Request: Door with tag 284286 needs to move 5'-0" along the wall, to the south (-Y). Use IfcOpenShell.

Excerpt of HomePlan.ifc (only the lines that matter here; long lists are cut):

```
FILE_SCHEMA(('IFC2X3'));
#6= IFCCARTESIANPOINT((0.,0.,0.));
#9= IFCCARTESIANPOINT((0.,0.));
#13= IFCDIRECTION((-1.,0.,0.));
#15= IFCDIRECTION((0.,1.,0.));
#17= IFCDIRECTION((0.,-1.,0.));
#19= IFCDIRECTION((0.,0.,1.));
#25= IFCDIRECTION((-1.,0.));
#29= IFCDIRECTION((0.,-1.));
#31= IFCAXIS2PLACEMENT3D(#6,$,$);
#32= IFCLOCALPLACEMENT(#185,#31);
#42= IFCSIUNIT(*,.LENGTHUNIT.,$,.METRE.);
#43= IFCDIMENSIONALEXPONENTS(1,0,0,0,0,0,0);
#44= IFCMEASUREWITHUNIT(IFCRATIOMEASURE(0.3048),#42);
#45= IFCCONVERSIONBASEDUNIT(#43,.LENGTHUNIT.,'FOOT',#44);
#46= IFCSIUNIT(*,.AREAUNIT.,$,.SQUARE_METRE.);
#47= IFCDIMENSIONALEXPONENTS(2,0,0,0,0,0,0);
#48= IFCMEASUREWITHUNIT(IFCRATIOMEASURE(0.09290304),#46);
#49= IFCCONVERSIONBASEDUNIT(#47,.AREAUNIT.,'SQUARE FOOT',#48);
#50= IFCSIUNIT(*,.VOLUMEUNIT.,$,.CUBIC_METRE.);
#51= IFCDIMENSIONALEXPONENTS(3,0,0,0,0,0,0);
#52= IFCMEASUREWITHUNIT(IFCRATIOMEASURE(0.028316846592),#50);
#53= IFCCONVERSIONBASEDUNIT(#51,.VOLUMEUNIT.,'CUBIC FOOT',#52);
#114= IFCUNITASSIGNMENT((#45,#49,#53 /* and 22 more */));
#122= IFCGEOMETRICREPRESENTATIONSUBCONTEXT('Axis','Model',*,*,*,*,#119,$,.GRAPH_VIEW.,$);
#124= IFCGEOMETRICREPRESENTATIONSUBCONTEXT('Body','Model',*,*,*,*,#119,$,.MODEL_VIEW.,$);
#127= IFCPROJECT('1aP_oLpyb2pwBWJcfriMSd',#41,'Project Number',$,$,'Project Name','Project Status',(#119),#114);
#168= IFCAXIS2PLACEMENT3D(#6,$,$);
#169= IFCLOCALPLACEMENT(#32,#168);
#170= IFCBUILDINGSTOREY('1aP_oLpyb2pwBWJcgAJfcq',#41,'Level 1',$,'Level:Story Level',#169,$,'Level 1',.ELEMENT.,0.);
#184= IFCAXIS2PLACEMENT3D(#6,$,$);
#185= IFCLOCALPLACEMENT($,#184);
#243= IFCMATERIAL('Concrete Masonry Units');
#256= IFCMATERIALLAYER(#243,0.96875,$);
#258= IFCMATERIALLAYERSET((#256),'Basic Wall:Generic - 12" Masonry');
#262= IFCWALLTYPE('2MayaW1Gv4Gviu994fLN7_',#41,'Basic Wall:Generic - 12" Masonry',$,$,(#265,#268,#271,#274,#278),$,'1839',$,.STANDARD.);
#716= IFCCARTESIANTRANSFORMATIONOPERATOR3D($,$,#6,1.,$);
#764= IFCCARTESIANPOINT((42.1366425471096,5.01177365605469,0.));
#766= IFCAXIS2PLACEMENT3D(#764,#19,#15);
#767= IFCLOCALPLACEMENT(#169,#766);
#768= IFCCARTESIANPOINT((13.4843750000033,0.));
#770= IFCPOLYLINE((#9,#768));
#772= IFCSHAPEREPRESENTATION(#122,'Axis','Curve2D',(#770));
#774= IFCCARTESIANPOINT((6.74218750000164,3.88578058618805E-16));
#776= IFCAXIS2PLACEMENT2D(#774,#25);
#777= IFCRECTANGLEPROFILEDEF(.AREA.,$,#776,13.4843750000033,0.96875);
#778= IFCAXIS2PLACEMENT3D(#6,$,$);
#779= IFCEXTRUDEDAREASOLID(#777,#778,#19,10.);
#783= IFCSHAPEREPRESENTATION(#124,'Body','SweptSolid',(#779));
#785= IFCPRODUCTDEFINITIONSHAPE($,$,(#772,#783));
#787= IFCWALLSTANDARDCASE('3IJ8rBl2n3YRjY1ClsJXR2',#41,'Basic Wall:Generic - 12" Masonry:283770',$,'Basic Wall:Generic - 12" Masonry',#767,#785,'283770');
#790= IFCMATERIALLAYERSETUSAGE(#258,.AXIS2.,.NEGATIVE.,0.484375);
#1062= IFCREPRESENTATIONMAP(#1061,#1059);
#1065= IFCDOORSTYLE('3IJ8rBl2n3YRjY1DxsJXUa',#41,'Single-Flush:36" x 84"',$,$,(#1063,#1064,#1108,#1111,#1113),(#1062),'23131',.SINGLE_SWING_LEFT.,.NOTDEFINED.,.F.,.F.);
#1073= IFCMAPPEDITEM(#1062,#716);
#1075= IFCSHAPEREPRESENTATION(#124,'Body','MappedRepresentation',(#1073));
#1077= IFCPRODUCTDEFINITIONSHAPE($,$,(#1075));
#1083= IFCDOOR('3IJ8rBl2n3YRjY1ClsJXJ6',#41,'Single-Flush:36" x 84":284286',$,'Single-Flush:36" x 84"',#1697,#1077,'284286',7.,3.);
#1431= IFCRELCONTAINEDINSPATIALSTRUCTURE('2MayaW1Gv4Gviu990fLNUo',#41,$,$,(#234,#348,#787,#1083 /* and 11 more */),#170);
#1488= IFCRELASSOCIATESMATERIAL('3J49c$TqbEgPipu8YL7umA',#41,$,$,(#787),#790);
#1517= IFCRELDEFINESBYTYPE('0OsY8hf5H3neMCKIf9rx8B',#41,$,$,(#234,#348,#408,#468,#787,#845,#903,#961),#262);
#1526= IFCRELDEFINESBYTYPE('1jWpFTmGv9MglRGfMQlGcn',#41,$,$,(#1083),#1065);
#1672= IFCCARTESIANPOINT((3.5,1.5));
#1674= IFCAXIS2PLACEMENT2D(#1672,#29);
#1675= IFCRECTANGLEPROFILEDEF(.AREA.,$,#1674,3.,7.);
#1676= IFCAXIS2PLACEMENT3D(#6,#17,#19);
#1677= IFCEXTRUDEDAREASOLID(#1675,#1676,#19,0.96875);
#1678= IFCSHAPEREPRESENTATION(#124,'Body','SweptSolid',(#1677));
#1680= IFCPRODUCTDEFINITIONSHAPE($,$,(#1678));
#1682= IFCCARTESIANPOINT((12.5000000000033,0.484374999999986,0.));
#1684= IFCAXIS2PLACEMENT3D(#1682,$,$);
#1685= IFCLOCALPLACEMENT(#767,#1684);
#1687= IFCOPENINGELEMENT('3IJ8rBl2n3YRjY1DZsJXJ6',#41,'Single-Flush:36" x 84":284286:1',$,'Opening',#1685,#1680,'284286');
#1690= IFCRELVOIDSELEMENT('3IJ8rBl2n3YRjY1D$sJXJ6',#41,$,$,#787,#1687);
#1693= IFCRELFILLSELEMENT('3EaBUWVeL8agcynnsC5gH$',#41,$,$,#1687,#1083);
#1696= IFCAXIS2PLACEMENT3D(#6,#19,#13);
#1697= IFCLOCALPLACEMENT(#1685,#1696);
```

```python
import ifcopenshell
import ifcopenshell.api.geometry
import ifcopenshell.util.placement
import ifcopenshell.util.unit

model = ifcopenshell.open("HomePlan.ifc")
unit_scale = ifcopenshell.util.unit.calculate_unit_scale(model)

door = model.by_guid("3IJ8rBl2n3YRjY1ClsJXJ6")
opening = door.FillsVoids[0].RelatingOpeningElement
wall = opening.VoidsElements[0].RelatingBuildingElement

wall_matrix = ifcopenshell.util.placement.get_local_placement(wall.ObjectPlacement)
shift = wall_matrix[:3, 0] * -60 * 0.0254 / unit_scale
before = ifcopenshell.util.placement.get_local_placement(door.ObjectPlacement)[:3, 3].copy()

# The door is placed relative to its opening, so it follows when the opening moves.
matrix = ifcopenshell.util.placement.get_local_placement(opening.ObjectPlacement)
matrix[:3, 3] += shift
ifcopenshell.api.geometry.edit_object_placement(
    model, product=opening, matrix=matrix, is_si=False, should_transform_children=True
)

after = ifcopenshell.util.placement.get_local_placement(door.ObjectPlacement)[:3, 3]
print("door moved by", (after - before).round(3) + 0.0)

model.write("HomePlan_edited.ifc")
```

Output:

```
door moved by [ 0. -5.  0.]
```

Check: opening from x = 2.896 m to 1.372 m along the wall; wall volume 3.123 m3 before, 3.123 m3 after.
